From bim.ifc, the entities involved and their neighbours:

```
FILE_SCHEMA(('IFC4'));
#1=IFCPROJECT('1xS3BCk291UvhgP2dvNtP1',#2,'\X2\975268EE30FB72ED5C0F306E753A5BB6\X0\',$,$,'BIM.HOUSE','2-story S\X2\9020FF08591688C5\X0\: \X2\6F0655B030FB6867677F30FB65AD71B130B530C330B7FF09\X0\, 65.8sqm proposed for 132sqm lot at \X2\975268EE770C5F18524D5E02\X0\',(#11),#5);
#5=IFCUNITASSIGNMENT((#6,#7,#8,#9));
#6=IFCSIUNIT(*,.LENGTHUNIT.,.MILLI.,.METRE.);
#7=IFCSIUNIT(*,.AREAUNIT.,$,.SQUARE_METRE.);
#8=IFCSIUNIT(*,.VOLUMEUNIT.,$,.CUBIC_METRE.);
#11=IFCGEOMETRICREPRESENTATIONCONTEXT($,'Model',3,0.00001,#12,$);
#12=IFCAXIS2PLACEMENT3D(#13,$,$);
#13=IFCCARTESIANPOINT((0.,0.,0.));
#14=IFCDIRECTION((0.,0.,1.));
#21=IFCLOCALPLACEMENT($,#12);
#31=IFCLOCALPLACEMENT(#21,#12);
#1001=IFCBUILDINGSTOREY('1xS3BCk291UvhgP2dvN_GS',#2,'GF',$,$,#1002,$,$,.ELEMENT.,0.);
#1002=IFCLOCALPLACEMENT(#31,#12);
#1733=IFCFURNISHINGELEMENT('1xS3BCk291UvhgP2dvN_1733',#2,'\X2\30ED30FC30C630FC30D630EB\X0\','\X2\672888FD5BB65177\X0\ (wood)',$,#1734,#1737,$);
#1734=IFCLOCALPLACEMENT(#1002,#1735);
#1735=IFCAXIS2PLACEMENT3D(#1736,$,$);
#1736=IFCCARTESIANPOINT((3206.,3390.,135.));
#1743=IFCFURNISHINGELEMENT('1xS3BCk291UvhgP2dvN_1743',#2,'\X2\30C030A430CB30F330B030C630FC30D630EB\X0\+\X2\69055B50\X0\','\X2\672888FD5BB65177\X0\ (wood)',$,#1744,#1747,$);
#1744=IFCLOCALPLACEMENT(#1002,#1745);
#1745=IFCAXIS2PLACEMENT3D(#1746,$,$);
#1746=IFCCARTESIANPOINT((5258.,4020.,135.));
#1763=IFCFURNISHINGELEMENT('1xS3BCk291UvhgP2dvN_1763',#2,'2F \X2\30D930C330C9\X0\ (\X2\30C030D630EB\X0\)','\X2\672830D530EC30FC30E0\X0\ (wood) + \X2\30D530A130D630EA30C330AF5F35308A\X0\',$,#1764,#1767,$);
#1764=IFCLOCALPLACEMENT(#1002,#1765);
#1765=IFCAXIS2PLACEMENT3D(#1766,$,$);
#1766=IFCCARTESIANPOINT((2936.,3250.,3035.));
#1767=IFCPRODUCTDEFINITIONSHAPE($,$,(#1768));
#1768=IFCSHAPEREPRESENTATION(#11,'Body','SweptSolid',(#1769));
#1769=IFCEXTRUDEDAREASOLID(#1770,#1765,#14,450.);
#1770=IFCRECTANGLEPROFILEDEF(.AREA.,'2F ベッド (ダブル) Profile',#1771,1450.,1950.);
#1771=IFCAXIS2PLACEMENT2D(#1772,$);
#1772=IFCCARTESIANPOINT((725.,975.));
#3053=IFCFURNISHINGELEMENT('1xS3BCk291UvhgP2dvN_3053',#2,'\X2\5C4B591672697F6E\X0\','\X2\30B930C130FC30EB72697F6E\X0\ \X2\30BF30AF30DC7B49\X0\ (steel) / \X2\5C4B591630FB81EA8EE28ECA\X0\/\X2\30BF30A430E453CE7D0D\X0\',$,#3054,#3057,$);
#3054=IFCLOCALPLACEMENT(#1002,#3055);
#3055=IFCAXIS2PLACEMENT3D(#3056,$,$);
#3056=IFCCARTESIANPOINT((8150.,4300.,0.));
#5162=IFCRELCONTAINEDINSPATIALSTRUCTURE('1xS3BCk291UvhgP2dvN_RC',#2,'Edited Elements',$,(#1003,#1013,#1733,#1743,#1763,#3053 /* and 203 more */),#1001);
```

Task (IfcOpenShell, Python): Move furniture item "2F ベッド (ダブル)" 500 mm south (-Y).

```python
import ifcopenshell
import ifcopenshell.api.geometry
import ifcopenshell.util.placement

model = ifcopenshell.open("bim.ifc")

item = model.by_guid("1xS3BCk291UvhgP2dvN_1763")
matrix = ifcopenshell.util.placement.get_local_placement(item.ObjectPlacement)
matrix[1, 3] -= 500.0
ifcopenshell.api.geometry.edit_object_placement(model, product=item, matrix=matrix, is_si=False)

print(ifcopenshell.util.placement.get_local_placement(item.ObjectPlacement).round(3) + 0.0)

model.write("bim_updated.ifc")
```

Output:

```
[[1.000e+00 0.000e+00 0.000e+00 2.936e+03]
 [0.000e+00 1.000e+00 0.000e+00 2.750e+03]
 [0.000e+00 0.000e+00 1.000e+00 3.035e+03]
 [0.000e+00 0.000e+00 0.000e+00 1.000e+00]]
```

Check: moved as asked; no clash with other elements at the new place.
